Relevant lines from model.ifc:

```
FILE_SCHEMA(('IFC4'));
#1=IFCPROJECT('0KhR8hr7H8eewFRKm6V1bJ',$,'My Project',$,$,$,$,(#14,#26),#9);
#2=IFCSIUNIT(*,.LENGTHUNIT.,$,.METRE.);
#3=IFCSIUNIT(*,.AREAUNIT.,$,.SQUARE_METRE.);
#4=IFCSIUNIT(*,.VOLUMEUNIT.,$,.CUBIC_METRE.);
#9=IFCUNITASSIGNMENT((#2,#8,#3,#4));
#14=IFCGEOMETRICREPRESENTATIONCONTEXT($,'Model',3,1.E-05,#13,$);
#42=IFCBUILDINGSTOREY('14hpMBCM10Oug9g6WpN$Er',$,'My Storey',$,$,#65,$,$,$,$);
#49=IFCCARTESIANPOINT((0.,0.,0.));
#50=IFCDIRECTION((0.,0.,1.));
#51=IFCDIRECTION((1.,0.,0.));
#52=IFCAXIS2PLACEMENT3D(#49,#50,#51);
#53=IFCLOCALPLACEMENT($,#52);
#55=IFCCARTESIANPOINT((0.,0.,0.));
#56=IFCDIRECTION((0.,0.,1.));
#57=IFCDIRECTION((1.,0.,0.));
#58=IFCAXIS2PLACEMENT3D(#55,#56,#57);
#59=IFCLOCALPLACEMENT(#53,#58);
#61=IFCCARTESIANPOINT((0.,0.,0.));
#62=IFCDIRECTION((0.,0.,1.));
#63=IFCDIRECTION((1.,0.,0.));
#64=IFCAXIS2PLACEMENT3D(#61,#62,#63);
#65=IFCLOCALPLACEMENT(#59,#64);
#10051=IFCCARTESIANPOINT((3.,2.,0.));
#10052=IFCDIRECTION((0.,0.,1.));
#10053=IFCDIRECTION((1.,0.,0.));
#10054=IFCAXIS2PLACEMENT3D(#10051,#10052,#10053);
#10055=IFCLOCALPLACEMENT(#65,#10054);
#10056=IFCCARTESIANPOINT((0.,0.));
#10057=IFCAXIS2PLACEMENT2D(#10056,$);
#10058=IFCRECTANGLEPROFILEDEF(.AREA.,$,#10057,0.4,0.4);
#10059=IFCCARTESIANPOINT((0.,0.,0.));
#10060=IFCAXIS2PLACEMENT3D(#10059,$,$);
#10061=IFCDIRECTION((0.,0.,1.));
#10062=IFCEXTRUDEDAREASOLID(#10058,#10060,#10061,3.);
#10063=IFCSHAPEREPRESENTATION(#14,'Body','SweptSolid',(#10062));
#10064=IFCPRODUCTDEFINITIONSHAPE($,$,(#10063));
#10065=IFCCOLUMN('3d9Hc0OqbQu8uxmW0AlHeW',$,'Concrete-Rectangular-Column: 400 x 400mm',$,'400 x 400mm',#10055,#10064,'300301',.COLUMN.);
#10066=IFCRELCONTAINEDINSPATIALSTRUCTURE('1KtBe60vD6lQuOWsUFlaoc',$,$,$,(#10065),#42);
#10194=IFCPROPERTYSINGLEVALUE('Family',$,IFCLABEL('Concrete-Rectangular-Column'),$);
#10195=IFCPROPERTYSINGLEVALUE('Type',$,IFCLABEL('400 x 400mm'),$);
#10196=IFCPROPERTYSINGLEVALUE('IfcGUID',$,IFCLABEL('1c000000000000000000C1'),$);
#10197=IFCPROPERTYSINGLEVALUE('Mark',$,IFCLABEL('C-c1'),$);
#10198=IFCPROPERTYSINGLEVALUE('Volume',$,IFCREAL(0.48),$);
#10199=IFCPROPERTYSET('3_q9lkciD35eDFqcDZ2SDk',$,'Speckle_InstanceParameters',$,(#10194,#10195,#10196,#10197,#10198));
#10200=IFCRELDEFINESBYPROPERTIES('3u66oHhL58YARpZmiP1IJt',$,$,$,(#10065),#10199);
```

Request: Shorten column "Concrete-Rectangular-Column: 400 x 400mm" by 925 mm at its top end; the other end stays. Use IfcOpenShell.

```python
import ifcopenshell
import ifcopenshell.api.pset
import ifcopenshell.util.element
import ifcopenshell.util.unit

model = ifcopenshell.open("model.ifc")
unit_scale = ifcopenshell.util.unit.calculate_unit_scale(model)

member = model.by_guid("3d9Hc0OqbQu8uxmW0AlHeW")
change = -0.925 / unit_scale

# The extrusion runs towards the end named, so only its depth changes.
body = next(r for r in member.Representation.Representations if r.RepresentationIdentifier == "Body")
solid = body.Items[0]
old_length = solid.Depth
solid.Depth += change

# Update the stored length and volume.
pset = model.by_id(ifcopenshell.util.element.get_pset(member, "Speckle_InstanceParameters", should_inherit=False)["id"])
ifcopenshell.api.pset.edit_pset(model, pset=pset, properties={
    "Volume": model.create_entity("IfcReal", ifcopenshell.util.element.get_pset(member, "Speckle_InstanceParameters", "Volume") * solid.Depth / old_length),
})

print(f"length {old_length:g} -> {solid.Depth:g}")

model.write("model-out.ifc")
```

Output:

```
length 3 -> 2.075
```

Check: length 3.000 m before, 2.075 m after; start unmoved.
